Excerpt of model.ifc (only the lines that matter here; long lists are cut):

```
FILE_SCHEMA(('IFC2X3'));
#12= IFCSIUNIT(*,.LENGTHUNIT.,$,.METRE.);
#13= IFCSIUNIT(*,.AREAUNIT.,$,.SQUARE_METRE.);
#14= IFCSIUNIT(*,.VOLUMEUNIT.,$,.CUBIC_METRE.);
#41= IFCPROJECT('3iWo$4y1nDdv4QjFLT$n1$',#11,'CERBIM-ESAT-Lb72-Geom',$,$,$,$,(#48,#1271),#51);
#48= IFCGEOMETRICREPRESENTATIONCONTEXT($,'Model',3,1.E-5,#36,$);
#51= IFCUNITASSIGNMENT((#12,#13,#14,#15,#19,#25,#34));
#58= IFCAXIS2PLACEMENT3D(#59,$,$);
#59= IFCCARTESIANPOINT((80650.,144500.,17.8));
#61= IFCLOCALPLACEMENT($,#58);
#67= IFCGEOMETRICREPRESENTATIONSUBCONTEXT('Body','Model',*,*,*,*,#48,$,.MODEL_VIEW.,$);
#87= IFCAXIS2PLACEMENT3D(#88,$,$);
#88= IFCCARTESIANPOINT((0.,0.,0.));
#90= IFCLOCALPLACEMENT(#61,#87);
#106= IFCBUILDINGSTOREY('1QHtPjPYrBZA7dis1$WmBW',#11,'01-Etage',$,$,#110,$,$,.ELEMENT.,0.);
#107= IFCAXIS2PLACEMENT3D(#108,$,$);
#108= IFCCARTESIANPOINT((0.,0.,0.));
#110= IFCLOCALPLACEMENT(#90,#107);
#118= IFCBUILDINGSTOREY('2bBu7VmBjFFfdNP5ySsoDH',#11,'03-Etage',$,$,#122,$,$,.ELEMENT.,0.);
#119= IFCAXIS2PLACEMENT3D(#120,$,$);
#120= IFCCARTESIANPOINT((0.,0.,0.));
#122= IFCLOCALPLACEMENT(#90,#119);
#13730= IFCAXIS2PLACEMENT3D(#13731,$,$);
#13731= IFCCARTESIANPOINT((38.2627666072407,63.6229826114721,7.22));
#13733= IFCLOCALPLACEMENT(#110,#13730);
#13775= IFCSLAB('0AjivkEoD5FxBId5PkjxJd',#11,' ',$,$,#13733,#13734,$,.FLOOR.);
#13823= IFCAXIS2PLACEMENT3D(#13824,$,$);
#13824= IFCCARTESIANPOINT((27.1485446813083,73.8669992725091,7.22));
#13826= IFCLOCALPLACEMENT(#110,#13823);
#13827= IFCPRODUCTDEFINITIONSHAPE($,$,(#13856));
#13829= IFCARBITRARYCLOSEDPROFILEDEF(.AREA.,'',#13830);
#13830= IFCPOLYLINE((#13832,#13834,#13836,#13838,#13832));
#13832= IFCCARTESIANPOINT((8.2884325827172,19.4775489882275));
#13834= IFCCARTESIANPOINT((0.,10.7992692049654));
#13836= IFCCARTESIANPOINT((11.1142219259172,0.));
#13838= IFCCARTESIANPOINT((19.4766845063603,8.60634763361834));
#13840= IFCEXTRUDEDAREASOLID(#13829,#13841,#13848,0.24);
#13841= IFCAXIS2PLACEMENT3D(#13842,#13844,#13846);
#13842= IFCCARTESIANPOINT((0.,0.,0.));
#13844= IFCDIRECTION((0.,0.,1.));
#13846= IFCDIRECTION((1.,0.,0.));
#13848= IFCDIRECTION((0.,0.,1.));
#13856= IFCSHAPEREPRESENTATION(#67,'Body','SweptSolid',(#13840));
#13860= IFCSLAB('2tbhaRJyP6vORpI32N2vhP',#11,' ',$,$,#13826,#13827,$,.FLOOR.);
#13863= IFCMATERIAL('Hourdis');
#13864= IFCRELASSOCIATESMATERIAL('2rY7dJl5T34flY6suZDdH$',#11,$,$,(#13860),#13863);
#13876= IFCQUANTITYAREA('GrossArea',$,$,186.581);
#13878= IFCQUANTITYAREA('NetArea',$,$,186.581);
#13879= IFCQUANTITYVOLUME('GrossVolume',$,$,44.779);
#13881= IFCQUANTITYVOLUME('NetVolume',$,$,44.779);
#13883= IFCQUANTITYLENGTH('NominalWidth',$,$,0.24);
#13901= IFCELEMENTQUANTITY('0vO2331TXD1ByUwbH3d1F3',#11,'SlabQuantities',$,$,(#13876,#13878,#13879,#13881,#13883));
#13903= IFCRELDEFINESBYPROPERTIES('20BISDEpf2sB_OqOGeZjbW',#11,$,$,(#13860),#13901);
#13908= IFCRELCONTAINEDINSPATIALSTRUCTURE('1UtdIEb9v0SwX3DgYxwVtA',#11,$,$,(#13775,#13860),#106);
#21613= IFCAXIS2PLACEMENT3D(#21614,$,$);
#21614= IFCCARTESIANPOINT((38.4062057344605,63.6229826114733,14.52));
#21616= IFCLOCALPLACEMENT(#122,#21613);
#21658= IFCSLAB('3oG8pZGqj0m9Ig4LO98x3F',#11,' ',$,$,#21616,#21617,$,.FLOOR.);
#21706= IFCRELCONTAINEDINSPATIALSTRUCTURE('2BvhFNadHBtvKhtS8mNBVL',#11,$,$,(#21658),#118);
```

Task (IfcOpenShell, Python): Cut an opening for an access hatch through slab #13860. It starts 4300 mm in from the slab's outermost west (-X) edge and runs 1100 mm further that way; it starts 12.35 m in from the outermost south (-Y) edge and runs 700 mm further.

```python
import numpy as np
import ifcopenshell
import ifcopenshell.api.feature
import ifcopenshell.api.geometry
import ifcopenshell.api.pset
import ifcopenshell.api.root
import ifcopenshell.geom
import ifcopenshell.util.element
import ifcopenshell.util.placement
import ifcopenshell.util.representation
import ifcopenshell.util.shape
import ifcopenshell.util.unit

model = ifcopenshell.open("model.ifc")
unit_scale = ifcopenshell.util.unit.calculate_unit_scale(model)
area_scale = ifcopenshell.util.unit.calculate_unit_scale(model, "AREAUNIT")
volume_scale = ifcopenshell.util.unit.calculate_unit_scale(model, "VOLUMEUNIT")
settings = ifcopenshell.geom.settings()


def volume(element):
    """Net volume in cubic metres, openings subtracted."""
    shape = ifcopenshell.geom.create_shape(settings, element)
    return ifcopenshell.util.shape.get_volume(shape.geometry)


slab = model.by_id(13860)
before = volume(slab)

# Extent in the slab's own axes, in metres. The edges named are its -X and -Y sides.
slab_shape = ifcopenshell.geom.create_shape(settings, slab)
vertices = ifcopenshell.util.shape.get_vertices(slab_shape.geometry)
x_min, y_min, bottom = vertices.min(axis=0)
top = vertices[:, 2].max()

opening = ifcopenshell.api.root.create_entity(model, ifc_class="IfcOpeningElement", name="Access hatch opening")
context = ifcopenshell.util.representation.get_context(model, "Model", "Body", "MODEL_VIEW")
width, depth = 1.1, 0.7
outline = [(0.0, 0.0), (width, 0.0), (width, depth), (0.0, depth), (0.0, 0.0)]
# Overshoot both faces by 50 mm so the cut is clean.
shape = ifcopenshell.api.geometry.add_slab_representation(
    model, context=context, depth=top - bottom + 0.1, polyline=outline
)
ifcopenshell.api.geometry.assign_representation(model, product=opening, representation=shape)

matrix = ifcopenshell.util.placement.get_local_placement(slab.ObjectPlacement)
matrix[:, 3] = matrix @ np.append(np.array([x_min + 4.3, y_min + 12.35, bottom - 0.05]) / unit_scale, 1.0)
ifcopenshell.api.geometry.edit_object_placement(model, product=opening, matrix=matrix, is_si=False)
ifcopenshell.api.feature.add_feature(model, feature=opening, element=slab)

after = volume(slab)

# Update the slab's stored quantities.
qto = model.by_id(ifcopenshell.util.element.get_pset(slab, "SlabQuantities", should_inherit=False)["id"])
ifcopenshell.api.pset.edit_qto(model, qto=qto, properties={
    "NetArea": after / (top - bottom) / area_scale,
    "NetVolume": after / volume_scale,
})

print(f"slab volume {before:.3f} -> {after:.3f} m3")

model.write("model_v2.ifc")
```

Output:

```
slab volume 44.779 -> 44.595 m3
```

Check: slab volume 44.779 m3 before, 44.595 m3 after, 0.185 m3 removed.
